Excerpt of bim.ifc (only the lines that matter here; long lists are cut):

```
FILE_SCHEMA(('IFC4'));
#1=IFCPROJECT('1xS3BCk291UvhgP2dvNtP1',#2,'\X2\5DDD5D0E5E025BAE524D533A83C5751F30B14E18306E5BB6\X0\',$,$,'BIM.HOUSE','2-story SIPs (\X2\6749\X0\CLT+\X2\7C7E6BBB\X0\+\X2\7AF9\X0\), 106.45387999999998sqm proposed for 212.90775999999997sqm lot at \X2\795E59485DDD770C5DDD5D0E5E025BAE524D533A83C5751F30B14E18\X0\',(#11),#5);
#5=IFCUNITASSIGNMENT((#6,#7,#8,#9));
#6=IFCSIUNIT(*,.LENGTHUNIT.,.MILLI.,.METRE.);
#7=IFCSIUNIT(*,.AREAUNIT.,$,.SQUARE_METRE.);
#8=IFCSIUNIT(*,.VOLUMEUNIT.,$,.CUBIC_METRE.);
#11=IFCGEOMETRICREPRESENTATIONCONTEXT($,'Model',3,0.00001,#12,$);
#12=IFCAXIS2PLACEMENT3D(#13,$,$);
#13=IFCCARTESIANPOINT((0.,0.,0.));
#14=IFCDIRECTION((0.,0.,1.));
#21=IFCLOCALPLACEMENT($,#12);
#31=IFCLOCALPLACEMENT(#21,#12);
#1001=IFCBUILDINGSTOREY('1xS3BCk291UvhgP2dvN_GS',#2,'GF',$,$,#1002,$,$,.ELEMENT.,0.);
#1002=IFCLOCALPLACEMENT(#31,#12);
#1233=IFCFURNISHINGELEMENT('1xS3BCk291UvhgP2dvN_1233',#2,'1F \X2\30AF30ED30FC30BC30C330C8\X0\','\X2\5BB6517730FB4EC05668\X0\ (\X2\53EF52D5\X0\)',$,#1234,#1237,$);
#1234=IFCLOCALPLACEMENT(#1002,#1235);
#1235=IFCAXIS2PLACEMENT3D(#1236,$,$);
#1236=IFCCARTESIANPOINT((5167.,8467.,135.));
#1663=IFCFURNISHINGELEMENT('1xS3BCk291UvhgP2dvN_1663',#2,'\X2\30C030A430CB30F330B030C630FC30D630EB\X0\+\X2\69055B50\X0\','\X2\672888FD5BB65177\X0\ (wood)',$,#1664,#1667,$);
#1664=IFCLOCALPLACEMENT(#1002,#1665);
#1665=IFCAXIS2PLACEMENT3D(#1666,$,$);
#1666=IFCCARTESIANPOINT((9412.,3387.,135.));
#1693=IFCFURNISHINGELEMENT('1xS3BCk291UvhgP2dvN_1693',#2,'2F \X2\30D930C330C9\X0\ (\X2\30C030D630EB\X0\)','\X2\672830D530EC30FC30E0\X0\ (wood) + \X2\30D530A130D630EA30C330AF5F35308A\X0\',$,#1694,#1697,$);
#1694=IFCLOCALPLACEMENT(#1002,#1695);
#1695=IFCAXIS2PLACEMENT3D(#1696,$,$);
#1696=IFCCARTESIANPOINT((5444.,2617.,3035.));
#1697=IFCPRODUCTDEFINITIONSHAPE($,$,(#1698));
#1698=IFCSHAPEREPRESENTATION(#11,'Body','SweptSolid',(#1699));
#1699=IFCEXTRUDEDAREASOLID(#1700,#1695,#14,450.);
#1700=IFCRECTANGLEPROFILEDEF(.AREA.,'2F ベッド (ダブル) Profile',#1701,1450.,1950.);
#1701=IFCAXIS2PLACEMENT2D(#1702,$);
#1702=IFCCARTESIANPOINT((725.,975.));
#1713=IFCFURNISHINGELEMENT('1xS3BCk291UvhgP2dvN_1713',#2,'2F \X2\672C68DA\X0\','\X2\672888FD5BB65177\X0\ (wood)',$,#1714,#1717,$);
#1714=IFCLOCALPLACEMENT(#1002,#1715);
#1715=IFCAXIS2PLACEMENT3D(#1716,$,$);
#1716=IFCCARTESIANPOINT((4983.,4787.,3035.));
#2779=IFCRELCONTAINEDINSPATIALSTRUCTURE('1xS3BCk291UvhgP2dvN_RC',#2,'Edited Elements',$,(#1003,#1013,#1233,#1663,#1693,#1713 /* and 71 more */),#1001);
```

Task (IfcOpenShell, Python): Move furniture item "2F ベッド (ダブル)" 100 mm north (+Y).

```python
import ifcopenshell
import ifcopenshell.api.geometry
import ifcopenshell.util.placement
import ifcopenshell.util.unit

model = ifcopenshell.open("bim.ifc")
unit_scale = ifcopenshell.util.unit.calculate_unit_scale(model)

item = model.by_id(1693)
matrix = ifcopenshell.util.placement.get_local_placement(item.ObjectPlacement)
matrix[1, 3] += 0.1 / unit_scale
ifcopenshell.api.geometry.edit_object_placement(model, product=item, matrix=matrix, is_si=False)

print(ifcopenshell.util.placement.get_local_placement(item.ObjectPlacement).round(3) + 0.0)

model.write("bim_edited.ifc")
```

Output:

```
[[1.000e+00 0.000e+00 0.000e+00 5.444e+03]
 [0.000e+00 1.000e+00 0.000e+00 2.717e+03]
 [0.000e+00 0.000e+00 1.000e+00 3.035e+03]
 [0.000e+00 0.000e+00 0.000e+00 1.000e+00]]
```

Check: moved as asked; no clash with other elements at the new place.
